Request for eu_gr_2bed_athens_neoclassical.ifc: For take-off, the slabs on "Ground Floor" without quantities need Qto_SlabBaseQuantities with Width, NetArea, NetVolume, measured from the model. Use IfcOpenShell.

First a look at what the model holds.

```python
import ifcopenshell
import ifcopenshell.util.element
import ifcopenshell.util.unit

model = ifcopenshell.open("eu_gr_2bed_athens_neoclassical.ifc")
print(model.schema)
for unit_type in ("LENGTHUNIT", "AREAUNIT", "VOLUMEUNIT"):
    print(unit_type, ifcopenshell.util.unit.calculate_unit_scale(model, unit_type))
storey = next(s for s in model.by_type("IfcBuildingStorey") if s.Name == "Ground Floor")
slabs = [e for e in ifcopenshell.util.element.get_decomposition(storey) if e.is_a("IfcSlab")]
for e in sorted(slabs, key=lambda e: e.id()):
    print(e.id(), e.is_a(), e.Name, list(ifcopenshell.util.element.get_psets(e, qtos_only=True)), sep=" | ")
```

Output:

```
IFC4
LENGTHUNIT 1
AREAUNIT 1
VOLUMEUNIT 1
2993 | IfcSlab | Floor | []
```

```python
import ifcopenshell
import ifcopenshell.api.pset
import ifcopenshell.geom
import ifcopenshell.util.element
import ifcopenshell.util.shape
import ifcopenshell.util.unit

model = ifcopenshell.open("eu_gr_2bed_athens_neoclassical.ifc")
unit_scale = ifcopenshell.util.unit.calculate_unit_scale(model)
area_scale = ifcopenshell.util.unit.calculate_unit_scale(model, "AREAUNIT")
volume_scale = ifcopenshell.util.unit.calculate_unit_scale(model, "VOLUMEUNIT")
settings = ifcopenshell.geom.settings()

storey = next(s for s in model.by_type("IfcBuildingStorey") if s.Name == "Ground Floor")
slabs = [e for e in ifcopenshell.util.element.get_decomposition(storey) if e.is_a("IfcSlab")]

for e in sorted(slabs, key=lambda e: e.id()):
    if ifcopenshell.util.element.get_psets(e, qtos_only=True, should_inherit=False):
        continue
    # Geometry comes back in metres, in the element's own axes.
    shape = ifcopenshell.geom.create_shape(settings, e)
    values = {
        "Width": ifcopenshell.util.shape.get_z(shape.geometry) / unit_scale,
        "NetArea": ifcopenshell.util.shape.get_footprint_area(shape.geometry) / area_scale,
        "NetVolume": ifcopenshell.util.shape.get_volume(shape.geometry) / volume_scale,
    }
    qto = ifcopenshell.api.pset.add_qto(model, product=e, name="Qto_SlabBaseQuantities")
    ifcopenshell.api.pset.edit_qto(model, qto=qto, properties=values)
    print(e.id(), {k: round(v, 3) for k, v in values.items()})

model.write("eu_gr_2bed_athens_neoclassical_v2.ifc")
```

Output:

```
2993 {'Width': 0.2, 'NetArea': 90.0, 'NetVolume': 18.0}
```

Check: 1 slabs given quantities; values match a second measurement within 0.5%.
